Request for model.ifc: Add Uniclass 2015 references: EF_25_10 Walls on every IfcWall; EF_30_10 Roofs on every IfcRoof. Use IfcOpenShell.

First a look at what the model holds.

```python
import ifcopenshell

model = ifcopenshell.open("model.ifc")
print(model.schema)
print("classifications:", [c.Name for c in model.by_type("IfcClassification")])
for ifc_class in ("IfcDoor", "IfcRoof", "IfcStair", "IfcWall", "IfcWindow"):
    print(ifc_class, len(model.by_type(ifc_class)))
```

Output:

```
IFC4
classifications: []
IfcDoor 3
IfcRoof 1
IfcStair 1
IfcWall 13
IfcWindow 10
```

```python
import ifcopenshell
import ifcopenshell.api.classification

model = ifcopenshell.open("model.ifc")

system = ifcopenshell.api.classification.add_classification(model, classification="Uniclass 2015")

codes = {
    "IfcWall": ("EF_25_10", "Walls"),
    "IfcRoof": ("EF_30_10", "Roofs"),
}
for ifc_class, (code, name) in codes.items():
    products = model.by_type(ifc_class)
    ifcopenshell.api.classification.add_reference(
        model, products=products, classification=system, identification=code, name=name
    )
    print(code, len(products))

model.write("model_rev.ifc")
```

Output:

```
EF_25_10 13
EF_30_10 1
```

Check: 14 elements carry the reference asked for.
